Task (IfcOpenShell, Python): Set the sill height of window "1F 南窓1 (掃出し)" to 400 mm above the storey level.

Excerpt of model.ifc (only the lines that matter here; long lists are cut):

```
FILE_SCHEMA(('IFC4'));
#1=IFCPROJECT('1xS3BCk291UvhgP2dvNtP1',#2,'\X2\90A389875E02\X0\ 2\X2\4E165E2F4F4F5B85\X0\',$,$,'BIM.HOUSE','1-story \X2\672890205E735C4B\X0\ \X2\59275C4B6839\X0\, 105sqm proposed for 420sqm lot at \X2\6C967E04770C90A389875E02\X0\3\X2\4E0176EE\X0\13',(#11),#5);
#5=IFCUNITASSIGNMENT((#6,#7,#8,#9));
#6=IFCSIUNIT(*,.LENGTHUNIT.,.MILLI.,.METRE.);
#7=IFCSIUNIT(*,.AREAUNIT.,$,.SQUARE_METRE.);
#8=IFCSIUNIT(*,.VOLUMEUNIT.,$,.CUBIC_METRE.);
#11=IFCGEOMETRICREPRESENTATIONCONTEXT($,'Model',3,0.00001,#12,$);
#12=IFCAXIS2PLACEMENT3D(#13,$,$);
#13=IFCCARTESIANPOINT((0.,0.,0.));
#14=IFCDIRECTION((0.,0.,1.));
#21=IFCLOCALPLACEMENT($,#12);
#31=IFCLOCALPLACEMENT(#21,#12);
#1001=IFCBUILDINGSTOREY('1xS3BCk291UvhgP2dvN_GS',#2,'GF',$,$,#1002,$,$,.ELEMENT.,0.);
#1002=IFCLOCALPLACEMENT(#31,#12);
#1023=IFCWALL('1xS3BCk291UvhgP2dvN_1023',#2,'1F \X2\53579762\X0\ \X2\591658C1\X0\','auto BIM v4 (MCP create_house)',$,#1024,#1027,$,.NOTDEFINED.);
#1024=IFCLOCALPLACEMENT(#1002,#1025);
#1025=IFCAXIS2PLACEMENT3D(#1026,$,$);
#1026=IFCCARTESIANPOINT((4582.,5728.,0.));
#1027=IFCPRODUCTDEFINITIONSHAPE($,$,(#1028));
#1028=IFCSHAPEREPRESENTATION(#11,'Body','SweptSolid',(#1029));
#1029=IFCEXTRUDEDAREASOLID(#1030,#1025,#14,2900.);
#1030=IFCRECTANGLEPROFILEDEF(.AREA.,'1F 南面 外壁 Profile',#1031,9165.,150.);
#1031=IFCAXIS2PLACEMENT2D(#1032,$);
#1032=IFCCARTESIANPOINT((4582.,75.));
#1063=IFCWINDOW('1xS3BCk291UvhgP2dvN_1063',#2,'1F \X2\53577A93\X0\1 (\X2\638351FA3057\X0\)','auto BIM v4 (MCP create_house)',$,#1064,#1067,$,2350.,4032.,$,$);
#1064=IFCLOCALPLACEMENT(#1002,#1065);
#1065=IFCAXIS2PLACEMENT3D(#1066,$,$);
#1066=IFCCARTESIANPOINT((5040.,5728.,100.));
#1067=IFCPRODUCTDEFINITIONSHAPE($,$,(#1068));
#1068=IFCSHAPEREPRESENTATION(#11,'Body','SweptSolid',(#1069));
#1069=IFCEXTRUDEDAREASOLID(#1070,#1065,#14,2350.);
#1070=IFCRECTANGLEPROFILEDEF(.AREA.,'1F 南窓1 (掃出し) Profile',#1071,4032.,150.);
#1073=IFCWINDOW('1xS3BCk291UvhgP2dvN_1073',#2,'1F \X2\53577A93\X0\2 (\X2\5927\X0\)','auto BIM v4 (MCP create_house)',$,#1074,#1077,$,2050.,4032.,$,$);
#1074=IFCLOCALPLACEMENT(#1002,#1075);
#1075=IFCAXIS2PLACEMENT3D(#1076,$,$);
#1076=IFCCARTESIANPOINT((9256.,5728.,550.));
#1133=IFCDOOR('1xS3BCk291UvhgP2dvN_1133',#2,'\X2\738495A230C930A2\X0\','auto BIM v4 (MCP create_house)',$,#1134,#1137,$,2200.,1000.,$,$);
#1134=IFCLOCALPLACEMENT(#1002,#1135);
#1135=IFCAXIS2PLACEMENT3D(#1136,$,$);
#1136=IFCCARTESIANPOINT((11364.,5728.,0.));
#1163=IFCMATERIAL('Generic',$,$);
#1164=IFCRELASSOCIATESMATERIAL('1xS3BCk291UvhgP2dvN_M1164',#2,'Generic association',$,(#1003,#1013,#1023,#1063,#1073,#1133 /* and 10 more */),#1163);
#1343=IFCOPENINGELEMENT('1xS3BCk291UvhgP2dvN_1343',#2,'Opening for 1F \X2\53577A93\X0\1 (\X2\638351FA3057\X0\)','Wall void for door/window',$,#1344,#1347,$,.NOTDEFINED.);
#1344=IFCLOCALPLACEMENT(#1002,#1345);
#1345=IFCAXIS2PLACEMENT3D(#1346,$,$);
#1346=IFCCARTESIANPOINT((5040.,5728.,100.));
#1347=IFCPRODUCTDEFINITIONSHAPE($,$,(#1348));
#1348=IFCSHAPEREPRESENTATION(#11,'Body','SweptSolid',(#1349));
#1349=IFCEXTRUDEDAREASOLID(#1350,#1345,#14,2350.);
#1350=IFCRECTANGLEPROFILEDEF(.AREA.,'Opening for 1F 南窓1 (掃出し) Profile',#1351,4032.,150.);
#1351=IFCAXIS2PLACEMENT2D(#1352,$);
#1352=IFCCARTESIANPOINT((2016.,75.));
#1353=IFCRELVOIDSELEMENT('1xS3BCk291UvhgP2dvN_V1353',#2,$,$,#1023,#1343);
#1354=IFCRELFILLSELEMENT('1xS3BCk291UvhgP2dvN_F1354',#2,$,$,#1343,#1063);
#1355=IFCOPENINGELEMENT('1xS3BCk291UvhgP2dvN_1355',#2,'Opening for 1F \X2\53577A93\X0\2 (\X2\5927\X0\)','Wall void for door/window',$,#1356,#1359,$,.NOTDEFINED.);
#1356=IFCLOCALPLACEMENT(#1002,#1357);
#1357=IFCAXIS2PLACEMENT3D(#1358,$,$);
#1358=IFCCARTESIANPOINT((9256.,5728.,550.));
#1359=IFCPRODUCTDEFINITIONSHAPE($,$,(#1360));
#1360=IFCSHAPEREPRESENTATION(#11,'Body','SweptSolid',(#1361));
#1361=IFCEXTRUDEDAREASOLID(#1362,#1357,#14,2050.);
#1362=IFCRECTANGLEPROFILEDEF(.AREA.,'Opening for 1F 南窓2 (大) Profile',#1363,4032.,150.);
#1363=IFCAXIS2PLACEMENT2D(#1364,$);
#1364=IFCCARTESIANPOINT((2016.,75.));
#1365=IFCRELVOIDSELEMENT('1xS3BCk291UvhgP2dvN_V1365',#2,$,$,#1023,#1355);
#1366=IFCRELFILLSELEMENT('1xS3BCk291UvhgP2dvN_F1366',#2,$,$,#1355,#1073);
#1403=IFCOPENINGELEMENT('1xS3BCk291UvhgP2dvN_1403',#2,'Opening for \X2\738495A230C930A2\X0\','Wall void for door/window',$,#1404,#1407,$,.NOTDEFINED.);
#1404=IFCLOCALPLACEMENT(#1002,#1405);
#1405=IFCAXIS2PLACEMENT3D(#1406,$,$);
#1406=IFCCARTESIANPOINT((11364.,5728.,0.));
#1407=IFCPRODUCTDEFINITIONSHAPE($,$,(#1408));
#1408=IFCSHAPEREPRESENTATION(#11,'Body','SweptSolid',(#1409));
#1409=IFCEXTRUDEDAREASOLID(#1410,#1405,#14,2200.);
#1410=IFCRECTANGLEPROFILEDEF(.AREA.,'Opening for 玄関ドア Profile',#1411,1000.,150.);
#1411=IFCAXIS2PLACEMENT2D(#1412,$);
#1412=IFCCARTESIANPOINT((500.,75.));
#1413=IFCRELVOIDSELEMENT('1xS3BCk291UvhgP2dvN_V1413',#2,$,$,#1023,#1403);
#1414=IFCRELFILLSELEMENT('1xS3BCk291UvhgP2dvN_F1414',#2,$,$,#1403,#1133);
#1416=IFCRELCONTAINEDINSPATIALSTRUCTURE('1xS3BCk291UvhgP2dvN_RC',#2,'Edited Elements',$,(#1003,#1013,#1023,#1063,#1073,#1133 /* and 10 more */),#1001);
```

```python
import numpy as np
import ifcopenshell
import ifcopenshell.api.geometry
import ifcopenshell.geom
import ifcopenshell.util.element
import ifcopenshell.util.placement
import ifcopenshell.util.shape
import ifcopenshell.util.unit

model = ifcopenshell.open("model.ifc")
unit_scale = ifcopenshell.util.unit.calculate_unit_scale(model)

window = model.by_guid("1xS3BCk291UvhgP2dvN_1063")
opening = window.FillsVoids[0].RelatingOpeningElement
storey = ifcopenshell.util.element.get_container(window, ifc_class="IfcBuildingStorey")
level = ifcopenshell.util.placement.get_local_placement(storey.ObjectPlacement)[2, 3]

# The opening's origin need not be at the sill, so measure its lowest point.
shape = ifcopenshell.geom.create_shape(ifcopenshell.geom.settings(), opening)
bottom = ifcopenshell.util.shape.get_shape_bottom_elevation(shape, shape.geometry) / unit_scale
dz = level + 0.4 / unit_scale - bottom

shift = np.array([0.0, 0.0, dz])
# The window is not placed relative to its opening, so move both.
for product in (opening, window):
    matrix = ifcopenshell.util.placement.get_local_placement(product.ObjectPlacement)
    matrix[:3, 3] += shift
    ifcopenshell.api.geometry.edit_object_placement(model, product=product, matrix=matrix, is_si=False)

print(f"moved by {dz * unit_scale:+.3f} m")

model.write("model_rev.ifc")
```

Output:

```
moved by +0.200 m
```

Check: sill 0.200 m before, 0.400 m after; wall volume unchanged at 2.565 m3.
